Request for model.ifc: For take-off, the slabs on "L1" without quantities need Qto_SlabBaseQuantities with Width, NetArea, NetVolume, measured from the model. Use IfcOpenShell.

First a look at what the model holds.

```python
import ifcopenshell
import ifcopenshell.util.element
import ifcopenshell.util.unit

model = ifcopenshell.open("model.ifc")
print(model.schema)
for unit_type in ("LENGTHUNIT", "AREAUNIT", "VOLUMEUNIT"):
    print(unit_type, ifcopenshell.util.unit.calculate_unit_scale(model, unit_type))
storey = next(s for s in model.by_type("IfcBuildingStorey") if s.Name == "L1")
slabs = [e for e in ifcopenshell.util.element.get_decomposition(storey) if e.is_a("IfcSlab")]
for e in sorted(slabs, key=lambda e: e.id()):
    print(e.id(), e.is_a(), e.Name, list(ifcopenshell.util.element.get_psets(e, qtos_only=True)), sep=" | ")
```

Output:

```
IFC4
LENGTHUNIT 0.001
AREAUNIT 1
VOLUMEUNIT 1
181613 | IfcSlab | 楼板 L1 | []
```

```python
import ifcopenshell
import ifcopenshell.api.pset
import ifcopenshell.geom
import ifcopenshell.util.element
import ifcopenshell.util.shape
import ifcopenshell.util.unit

model = ifcopenshell.open("model.ifc")
unit_scale = ifcopenshell.util.unit.calculate_unit_scale(model)
area_scale = ifcopenshell.util.unit.calculate_unit_scale(model, "AREAUNIT")
volume_scale = ifcopenshell.util.unit.calculate_unit_scale(model, "VOLUMEUNIT")
settings = ifcopenshell.geom.settings()

storey = next(s for s in model.by_type("IfcBuildingStorey") if s.Name == "L1")
slabs = [e for e in ifcopenshell.util.element.get_decomposition(storey) if e.is_a("IfcSlab")]

for e in sorted(slabs, key=lambda e: e.id()):
    if ifcopenshell.util.element.get_psets(e, qtos_only=True, should_inherit=False):
        continue
    # Geometry comes back in metres, in the element's own axes.
    shape = ifcopenshell.geom.create_shape(settings, e)
    values = {
        "Width": ifcopenshell.util.shape.get_z(shape.geometry) / unit_scale,
        "NetArea": ifcopenshell.util.shape.get_footprint_area(shape.geometry) / area_scale,
        "NetVolume": ifcopenshell.util.shape.get_volume(shape.geometry) / volume_scale,
    }
    qto = ifcopenshell.api.pset.add_qto(model, product=e, name="Qto_SlabBaseQuantities")
    ifcopenshell.api.pset.edit_qto(model, qto=qto, properties=values)
    print(e.id(), {k: round(v, 3) for k, v in values.items()})

model.write("model_v2.ifc")
```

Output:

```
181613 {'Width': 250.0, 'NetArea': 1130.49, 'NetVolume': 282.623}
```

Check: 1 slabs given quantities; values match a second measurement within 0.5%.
